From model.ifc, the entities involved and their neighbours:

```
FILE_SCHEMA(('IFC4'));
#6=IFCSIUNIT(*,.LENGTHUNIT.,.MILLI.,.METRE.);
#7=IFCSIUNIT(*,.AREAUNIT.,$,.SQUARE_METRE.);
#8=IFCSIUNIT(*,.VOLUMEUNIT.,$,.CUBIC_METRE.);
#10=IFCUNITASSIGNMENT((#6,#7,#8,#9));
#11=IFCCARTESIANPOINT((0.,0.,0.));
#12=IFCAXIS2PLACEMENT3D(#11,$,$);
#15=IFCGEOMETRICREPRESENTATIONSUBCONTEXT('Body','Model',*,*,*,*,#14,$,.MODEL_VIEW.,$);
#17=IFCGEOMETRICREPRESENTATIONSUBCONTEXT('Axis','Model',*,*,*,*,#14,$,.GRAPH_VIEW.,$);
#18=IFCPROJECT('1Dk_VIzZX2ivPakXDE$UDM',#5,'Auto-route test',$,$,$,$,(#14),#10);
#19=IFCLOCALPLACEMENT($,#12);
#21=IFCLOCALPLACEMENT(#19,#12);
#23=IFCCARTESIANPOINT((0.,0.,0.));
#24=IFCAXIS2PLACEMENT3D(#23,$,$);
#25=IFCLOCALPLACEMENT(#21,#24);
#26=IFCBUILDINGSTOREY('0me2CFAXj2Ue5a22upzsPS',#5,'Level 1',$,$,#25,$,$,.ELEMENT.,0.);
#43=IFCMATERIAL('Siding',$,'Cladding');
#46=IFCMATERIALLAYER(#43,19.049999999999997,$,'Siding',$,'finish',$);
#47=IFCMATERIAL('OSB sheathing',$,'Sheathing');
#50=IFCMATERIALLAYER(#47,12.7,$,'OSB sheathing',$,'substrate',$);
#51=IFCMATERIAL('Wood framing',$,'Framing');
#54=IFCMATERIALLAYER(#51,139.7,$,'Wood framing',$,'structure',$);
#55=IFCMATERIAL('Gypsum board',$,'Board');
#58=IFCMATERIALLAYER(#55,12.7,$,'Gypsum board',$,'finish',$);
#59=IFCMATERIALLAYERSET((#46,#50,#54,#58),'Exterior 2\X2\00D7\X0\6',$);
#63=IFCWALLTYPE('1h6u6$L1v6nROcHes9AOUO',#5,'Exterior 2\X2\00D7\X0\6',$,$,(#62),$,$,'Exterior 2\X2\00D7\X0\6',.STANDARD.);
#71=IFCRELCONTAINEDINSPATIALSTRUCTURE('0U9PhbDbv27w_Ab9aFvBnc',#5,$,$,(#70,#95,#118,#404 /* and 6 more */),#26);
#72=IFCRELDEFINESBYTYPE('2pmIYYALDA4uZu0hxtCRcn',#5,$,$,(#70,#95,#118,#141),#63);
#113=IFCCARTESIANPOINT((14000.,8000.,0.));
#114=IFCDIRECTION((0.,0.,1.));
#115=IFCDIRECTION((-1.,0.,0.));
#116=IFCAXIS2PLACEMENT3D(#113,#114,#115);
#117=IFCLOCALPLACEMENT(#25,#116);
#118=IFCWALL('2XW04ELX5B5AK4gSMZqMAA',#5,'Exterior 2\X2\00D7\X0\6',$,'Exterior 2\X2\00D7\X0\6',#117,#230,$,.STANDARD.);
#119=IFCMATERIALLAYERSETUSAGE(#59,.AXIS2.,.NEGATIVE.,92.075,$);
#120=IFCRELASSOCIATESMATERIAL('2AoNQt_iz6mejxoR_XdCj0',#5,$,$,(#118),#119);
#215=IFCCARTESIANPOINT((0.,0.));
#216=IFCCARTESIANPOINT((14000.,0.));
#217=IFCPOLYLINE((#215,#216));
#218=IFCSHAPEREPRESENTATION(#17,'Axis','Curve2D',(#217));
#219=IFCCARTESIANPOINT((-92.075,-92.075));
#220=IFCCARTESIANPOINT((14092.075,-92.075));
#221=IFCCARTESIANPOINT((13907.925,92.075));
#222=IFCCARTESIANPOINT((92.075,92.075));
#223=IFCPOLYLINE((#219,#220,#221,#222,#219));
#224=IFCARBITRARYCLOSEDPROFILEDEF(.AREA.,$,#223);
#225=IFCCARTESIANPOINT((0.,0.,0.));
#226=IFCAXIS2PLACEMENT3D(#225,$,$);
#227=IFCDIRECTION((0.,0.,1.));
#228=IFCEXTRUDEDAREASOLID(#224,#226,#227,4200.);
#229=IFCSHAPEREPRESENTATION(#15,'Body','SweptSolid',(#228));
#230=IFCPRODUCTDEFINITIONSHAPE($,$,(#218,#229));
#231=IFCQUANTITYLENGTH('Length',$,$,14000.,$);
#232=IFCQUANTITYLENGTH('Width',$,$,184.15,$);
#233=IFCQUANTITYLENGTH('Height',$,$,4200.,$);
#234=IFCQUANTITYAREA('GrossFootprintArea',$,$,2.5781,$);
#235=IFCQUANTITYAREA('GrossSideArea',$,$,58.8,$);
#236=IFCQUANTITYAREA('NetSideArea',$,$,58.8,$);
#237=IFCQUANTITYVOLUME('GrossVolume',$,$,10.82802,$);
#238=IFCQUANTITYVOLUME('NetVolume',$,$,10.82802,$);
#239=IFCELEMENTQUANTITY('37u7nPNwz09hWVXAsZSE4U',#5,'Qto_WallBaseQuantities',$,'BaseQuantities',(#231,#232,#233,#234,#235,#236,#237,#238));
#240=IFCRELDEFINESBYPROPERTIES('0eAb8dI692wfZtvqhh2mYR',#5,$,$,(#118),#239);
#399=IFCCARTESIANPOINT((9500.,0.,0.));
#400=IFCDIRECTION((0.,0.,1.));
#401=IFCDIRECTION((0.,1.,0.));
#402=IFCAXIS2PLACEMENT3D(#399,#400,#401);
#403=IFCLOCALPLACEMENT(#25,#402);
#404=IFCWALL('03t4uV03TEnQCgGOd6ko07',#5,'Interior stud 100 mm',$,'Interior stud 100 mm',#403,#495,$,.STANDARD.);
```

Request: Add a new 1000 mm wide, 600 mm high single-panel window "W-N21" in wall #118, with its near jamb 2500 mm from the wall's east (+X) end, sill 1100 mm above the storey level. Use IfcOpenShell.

```python
import numpy as np
import ifcopenshell
import ifcopenshell.api.feature
import ifcopenshell.api.geometry
import ifcopenshell.api.pset
import ifcopenshell.api.root
import ifcopenshell.api.spatial
import ifcopenshell.geom
import ifcopenshell.util.element
import ifcopenshell.util.placement
import ifcopenshell.util.representation
import ifcopenshell.util.shape
import ifcopenshell.util.unit

model = ifcopenshell.open("model.ifc")
unit_scale = ifcopenshell.util.unit.calculate_unit_scale(model)
area_scale = ifcopenshell.util.unit.calculate_unit_scale(model, "AREAUNIT")
volume_scale = ifcopenshell.util.unit.calculate_unit_scale(model, "VOLUMEUNIT")
settings = ifcopenshell.geom.settings()


def volume(element):
    """Net volume in cubic metres, openings subtracted."""
    shape = ifcopenshell.geom.create_shape(settings, element)
    return ifcopenshell.util.shape.get_volume(shape.geometry)


wall = model.by_guid("2XW04ELX5B5AK4gSMZqMAA")
storey = ifcopenshell.util.element.get_container(wall, ifc_class="IfcBuildingStorey")
context = ifcopenshell.util.representation.get_context(model, "Model", "Body", "MODEL_VIEW")
before = volume(wall)

width, height, from_end, sill = 1, 0.6, 2.5, 1.1  # metres

# The wall runs along its own X axis, and the end named is its -X end.
wall_shape = ifcopenshell.geom.create_shape(settings, wall)
x, y, z = ifcopenshell.util.shape.get_vertices(wall_shape.geometry).T
start = x.min() + from_end
face, thickness = float(y.min()), float(y.max() - y.min())
wall_matrix = ifcopenshell.util.placement.get_local_placement(wall.ObjectPlacement)
level = ifcopenshell.util.placement.get_local_placement(storey.ObjectPlacement)[2, 3]


def in_wall(x, y):
    """Placement at x, y metres in the wall's axes, at sill height."""
    matrix = wall_matrix.copy()
    matrix[:, 3] = wall_matrix @ np.array([x / unit_scale, y / unit_scale, 0.0, 1.0])
    matrix[2, 3] = level + sill / unit_scale
    return matrix


# Opening: a box that overshoots both wall faces by 50 mm.
opening = ifcopenshell.api.root.create_entity(model, ifc_class="IfcOpeningElement", predefined_type="OPENING")
box = ifcopenshell.api.geometry.add_wall_representation(
    model, context=context, length=width, height=height, thickness=thickness + 0.1
)
ifcopenshell.api.geometry.assign_representation(model, product=opening, representation=box)
ifcopenshell.api.geometry.edit_object_placement(model, product=opening, matrix=in_wall(start, face - 0.05), is_si=False)
ifcopenshell.api.feature.add_feature(model, feature=opening, element=wall)

window = ifcopenshell.api.root.create_entity(model, ifc_class="IfcWindow", name="W-N21", predefined_type="WINDOW")
window.OverallWidth, window.OverallHeight = width / unit_scale, height / unit_scale
window.PartitioningType = "SINGLE_PANEL"
body = ifcopenshell.api.geometry.add_window_representation(
    model,
    context=context,
    overall_width=window.OverallWidth,
    overall_height=window.OverallHeight,
    partition_type="SINGLE_PANEL",
)
ifcopenshell.api.geometry.assign_representation(model, product=window, representation=body)
ifcopenshell.api.spatial.assign_container(model, products=[window], relating_structure=storey)
ifcopenshell.api.feature.add_filling(model, opening=opening, element=window)

# Centre the window in the wall's thickness.
ifcopenshell.api.geometry.edit_object_placement(model, product=window, matrix=in_wall(start, face), is_si=False)
window_shape = ifcopenshell.geom.create_shape(settings, window)
depth = ifcopenshell.util.shape.get_vertices(window_shape.geometry)[:, 1]
offset = face + thickness / 2 - (depth.min() + depth.max()) / 2
ifcopenshell.api.geometry.edit_object_placement(model, product=window, matrix=in_wall(start, offset), is_si=False)

after = volume(wall)

# Update the wall's stored quantities.
qto = model.by_id(ifcopenshell.util.element.get_pset(wall, "Qto_WallBaseQuantities", should_inherit=False)["id"])
ifcopenshell.api.pset.edit_qto(model, qto=qto, properties={
    "NetSideArea": after / thickness / area_scale,
    "NetVolume": after / volume_scale,
})

print(f"wall volume {before:.3f} -> {after:.3f} m3")

model.write("model_edited.ifc")
```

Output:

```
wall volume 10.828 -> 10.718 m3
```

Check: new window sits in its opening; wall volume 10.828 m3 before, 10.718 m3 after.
